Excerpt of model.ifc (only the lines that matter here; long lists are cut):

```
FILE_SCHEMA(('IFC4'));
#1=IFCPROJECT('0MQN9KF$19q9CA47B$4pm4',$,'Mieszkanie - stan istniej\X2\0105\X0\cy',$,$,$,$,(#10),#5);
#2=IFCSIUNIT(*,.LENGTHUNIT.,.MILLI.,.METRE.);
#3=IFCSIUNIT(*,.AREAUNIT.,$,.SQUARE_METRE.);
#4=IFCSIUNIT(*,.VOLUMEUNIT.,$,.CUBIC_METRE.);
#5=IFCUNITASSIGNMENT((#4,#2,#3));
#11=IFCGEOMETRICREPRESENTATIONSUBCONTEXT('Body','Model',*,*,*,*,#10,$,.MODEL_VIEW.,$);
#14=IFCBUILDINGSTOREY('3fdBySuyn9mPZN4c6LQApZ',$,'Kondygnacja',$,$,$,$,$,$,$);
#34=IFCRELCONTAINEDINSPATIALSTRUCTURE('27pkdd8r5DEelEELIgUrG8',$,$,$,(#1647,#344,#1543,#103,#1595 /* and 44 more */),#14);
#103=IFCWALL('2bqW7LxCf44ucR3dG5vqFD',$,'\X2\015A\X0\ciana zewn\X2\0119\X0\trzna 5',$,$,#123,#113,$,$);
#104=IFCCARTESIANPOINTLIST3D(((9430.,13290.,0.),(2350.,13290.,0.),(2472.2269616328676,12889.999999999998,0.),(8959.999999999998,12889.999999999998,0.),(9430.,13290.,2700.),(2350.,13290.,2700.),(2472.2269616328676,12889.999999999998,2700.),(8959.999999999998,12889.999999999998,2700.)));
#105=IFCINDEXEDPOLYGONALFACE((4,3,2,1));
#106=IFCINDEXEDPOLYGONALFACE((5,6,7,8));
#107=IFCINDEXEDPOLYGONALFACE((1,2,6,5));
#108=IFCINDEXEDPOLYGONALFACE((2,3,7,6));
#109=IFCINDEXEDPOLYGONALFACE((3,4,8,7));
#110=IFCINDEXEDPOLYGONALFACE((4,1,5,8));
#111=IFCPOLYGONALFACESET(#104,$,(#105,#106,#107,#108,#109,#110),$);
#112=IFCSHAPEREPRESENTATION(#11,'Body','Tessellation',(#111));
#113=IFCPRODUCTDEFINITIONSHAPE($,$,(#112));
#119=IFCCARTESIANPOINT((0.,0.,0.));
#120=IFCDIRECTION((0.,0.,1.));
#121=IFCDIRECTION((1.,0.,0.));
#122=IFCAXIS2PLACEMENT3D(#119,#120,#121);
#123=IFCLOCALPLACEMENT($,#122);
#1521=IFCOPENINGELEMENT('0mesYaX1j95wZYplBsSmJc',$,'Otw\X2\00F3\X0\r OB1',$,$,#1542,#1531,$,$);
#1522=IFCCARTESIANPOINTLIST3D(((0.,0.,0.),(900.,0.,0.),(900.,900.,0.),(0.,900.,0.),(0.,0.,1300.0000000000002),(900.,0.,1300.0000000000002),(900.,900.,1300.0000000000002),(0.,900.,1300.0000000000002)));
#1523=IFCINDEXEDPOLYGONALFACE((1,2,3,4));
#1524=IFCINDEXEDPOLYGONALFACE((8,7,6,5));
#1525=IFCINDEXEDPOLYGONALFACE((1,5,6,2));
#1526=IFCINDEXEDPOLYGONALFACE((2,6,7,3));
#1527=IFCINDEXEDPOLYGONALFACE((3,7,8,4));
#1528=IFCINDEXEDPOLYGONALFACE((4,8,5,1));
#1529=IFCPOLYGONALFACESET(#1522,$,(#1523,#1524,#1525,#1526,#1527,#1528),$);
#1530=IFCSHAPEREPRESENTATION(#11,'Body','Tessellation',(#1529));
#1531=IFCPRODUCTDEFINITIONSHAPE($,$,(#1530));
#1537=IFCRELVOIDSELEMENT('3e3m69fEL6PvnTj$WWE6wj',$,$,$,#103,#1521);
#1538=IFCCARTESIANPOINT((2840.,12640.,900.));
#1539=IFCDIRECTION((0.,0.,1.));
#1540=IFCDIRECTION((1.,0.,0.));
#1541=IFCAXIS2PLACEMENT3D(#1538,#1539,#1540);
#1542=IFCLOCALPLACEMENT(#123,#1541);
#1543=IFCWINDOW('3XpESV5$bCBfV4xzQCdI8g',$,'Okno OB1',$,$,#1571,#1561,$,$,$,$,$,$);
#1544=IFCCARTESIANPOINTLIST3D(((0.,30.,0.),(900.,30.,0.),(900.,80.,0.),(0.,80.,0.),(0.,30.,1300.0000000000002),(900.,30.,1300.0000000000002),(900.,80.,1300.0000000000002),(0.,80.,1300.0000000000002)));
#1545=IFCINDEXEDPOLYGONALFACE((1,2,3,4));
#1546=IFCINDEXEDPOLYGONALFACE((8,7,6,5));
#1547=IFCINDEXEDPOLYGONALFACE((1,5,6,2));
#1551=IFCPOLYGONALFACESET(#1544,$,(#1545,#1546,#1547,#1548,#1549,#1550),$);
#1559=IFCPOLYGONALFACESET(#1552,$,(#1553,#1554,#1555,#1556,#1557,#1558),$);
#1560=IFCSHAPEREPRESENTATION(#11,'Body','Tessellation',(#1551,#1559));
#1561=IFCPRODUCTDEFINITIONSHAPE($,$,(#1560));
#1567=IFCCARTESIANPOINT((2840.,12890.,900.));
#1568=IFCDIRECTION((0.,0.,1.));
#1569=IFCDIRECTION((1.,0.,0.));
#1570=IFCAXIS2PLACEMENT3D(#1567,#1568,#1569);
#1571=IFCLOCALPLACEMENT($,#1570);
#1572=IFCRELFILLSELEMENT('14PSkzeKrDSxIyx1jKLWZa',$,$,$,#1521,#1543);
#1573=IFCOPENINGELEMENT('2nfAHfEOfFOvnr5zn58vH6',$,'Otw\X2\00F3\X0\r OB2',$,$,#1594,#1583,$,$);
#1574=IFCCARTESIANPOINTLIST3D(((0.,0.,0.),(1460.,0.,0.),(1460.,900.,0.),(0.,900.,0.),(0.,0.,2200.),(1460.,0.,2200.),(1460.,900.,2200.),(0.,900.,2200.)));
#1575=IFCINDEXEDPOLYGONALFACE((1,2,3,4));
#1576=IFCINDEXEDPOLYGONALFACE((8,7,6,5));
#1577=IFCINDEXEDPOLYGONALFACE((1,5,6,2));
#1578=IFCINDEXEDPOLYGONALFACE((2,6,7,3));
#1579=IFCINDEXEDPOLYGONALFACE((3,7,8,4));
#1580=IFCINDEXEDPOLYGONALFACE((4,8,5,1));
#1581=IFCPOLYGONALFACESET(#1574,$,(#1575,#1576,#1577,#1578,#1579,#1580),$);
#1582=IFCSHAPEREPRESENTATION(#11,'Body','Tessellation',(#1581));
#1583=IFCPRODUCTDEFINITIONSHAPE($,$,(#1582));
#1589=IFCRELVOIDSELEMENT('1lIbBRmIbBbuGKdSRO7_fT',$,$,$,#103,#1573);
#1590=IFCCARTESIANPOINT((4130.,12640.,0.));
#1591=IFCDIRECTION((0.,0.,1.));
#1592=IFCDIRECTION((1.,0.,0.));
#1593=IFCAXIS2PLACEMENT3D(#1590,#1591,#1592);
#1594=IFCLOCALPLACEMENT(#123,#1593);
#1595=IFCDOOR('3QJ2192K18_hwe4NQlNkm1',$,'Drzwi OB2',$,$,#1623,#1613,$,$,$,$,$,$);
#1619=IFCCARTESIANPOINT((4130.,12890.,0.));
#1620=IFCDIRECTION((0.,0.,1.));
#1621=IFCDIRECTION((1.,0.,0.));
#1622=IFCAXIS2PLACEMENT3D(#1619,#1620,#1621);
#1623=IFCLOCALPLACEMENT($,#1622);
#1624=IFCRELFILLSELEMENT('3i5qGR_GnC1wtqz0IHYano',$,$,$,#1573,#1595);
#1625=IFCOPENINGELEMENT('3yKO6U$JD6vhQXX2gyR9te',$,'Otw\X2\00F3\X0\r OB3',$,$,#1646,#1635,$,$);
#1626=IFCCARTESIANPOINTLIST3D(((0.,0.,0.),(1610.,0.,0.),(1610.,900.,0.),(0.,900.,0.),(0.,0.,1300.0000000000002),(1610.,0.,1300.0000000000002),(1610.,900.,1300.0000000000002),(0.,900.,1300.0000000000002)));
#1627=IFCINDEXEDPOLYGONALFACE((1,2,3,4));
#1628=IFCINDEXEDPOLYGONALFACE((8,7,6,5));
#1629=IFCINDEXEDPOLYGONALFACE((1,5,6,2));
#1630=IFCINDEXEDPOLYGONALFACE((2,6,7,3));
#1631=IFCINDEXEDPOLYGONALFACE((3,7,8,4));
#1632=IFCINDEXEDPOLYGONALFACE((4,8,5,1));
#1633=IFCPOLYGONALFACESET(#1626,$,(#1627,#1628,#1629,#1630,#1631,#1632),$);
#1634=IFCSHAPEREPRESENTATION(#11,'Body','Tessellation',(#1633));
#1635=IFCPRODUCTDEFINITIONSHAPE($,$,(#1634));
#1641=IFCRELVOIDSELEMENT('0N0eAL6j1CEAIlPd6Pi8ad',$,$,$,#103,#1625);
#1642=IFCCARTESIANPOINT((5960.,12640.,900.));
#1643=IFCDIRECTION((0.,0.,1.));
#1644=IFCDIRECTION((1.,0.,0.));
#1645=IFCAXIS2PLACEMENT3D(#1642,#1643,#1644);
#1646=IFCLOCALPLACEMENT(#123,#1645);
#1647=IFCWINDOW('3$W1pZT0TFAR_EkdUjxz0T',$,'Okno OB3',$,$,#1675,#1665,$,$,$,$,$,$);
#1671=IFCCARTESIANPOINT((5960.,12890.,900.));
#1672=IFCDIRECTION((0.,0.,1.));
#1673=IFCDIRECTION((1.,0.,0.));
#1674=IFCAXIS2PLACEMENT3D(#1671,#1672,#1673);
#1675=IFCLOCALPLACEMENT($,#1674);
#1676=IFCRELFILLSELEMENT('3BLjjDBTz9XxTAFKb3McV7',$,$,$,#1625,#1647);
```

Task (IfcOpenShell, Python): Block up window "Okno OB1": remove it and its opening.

```python
import ifcopenshell
import ifcopenshell.api.feature
import ifcopenshell.api.root
import ifcopenshell.geom
import ifcopenshell.util.shape

model = ifcopenshell.open("model.ifc")
settings = ifcopenshell.geom.settings()


def volume(element):
    """Net volume in cubic metres, openings subtracted."""
    shape = ifcopenshell.geom.create_shape(settings, element)
    return ifcopenshell.util.shape.get_volume(shape.geometry)


window = model.by_guid("3XpESV5$bCBfV4xzQCdI8g")
opening = window.FillsVoids[0].RelatingOpeningElement
wall = opening.VoidsElements[0].RelatingBuildingElement
before = volume(wall)

ifcopenshell.api.root.remove_product(model, product=window)
ifcopenshell.api.feature.remove_feature(model, feature=opening)

after = volume(wall)

print(f"wall volume {before:.3f} -> {after:.3f} m3")

model.write("model-out.ifc")
```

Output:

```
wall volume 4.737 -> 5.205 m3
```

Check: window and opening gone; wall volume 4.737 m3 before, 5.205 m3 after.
